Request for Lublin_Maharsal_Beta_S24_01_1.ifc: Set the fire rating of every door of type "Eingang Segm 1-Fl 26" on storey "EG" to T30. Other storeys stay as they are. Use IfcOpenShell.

First a look at what the model holds.

```python
import ifcopenshell
import ifcopenshell.util.element

model = ifcopenshell.open("Lublin_Maharsal_Beta_S24_01_1.ifc")
print(model.schema)
storey = next(s for s in model.by_type("IfcBuildingStorey") if s.Name == "EG")
doors = [e for e in ifcopenshell.util.element.get_decomposition(storey) if e.is_a("IfcDoor")]
seen = {}
for e in doors:
    element_type = ifcopenshell.util.element.get_type(e)
    key = (element_type.Name if element_type != e and element_type else None, ifcopenshell.util.element.get_pset(e, "Pset_DoorCommon", "FireRating"))
    seen[key] = seen.get(key, 0) + 1
for (name, value), count in sorted(seen.items(), key=str):
    print(count, "x", name, "|", value)
```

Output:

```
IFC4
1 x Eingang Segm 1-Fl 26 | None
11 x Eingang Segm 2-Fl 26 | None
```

```python
import ifcopenshell
import ifcopenshell.api.pset
import ifcopenshell.util.element

model = ifcopenshell.open("Lublin_Maharsal_Beta_S24_01_1.ifc")

storey = next(s for s in model.by_type("IfcBuildingStorey") if s.Name == "EG")
doors = [e for e in ifcopenshell.util.element.get_decomposition(storey) if e.is_a("IfcDoor")]

count = 0
for e in doors:
    element_type = ifcopenshell.util.element.get_type(e)
    if element_type in (None, e) or element_type.Name != "Eingang Segm 1-Fl 26":
        continue
    # add_pset returns the element's existing set when there is one.
    pset = ifcopenshell.api.pset.add_pset(model, product=e, name="Pset_DoorCommon")
    ifcopenshell.api.pset.edit_pset(model, pset=pset, properties={"FireRating": "T30"})
    count += 1

print(count, "doors updated")

model.write("Lublin_Maharsal_Beta_S24_01_1_edited.ifc")
```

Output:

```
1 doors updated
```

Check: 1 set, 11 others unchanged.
